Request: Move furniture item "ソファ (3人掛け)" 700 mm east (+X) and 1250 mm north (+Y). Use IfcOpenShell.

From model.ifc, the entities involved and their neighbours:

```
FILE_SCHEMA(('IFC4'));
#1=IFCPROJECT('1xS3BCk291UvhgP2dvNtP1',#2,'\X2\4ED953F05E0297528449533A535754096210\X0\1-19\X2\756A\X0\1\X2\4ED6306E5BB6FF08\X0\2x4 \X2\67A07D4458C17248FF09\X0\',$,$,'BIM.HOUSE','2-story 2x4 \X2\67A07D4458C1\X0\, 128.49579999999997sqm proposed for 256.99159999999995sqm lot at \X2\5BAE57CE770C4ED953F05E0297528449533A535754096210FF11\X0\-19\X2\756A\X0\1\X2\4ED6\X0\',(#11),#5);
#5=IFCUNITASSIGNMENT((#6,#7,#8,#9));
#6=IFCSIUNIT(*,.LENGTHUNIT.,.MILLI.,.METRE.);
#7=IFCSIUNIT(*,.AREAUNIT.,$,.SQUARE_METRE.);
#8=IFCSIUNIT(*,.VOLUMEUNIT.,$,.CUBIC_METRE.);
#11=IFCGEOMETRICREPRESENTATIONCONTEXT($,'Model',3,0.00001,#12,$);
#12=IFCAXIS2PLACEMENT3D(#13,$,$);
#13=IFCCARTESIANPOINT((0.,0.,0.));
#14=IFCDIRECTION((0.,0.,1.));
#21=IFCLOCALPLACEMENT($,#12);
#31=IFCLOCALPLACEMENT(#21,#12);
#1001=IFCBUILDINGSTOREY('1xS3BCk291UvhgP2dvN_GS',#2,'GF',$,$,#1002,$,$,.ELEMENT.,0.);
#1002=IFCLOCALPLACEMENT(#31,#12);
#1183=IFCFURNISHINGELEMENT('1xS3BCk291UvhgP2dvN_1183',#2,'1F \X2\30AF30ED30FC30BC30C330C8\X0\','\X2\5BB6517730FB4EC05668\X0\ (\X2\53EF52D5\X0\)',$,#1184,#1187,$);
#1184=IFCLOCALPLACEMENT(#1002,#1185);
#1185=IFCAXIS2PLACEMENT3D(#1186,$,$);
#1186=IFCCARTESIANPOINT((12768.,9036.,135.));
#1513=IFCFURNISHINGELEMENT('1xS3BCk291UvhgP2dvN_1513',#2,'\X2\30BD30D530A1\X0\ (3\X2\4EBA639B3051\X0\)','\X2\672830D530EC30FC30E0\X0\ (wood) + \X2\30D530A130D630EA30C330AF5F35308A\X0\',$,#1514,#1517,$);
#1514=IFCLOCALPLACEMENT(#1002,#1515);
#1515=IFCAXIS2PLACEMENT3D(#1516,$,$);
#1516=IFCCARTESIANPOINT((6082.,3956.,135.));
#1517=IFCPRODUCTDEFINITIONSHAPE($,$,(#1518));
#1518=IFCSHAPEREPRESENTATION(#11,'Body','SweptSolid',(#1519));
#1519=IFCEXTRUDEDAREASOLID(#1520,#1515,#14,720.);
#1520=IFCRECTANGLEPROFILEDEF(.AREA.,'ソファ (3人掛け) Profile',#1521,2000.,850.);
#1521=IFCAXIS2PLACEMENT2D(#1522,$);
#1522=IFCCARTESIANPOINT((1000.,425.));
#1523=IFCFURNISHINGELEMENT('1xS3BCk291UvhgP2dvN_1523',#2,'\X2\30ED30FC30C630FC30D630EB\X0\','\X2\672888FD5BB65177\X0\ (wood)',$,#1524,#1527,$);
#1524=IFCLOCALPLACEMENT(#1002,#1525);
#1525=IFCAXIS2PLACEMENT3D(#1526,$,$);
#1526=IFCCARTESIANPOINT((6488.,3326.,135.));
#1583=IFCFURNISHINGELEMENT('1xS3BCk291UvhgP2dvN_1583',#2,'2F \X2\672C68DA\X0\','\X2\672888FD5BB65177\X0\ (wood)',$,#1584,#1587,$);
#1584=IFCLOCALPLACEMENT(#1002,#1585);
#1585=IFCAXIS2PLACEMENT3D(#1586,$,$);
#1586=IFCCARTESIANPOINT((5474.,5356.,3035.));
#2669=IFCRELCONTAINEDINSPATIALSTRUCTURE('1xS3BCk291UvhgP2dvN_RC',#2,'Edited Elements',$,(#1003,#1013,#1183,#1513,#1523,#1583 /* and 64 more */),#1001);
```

```python
import ifcopenshell
import ifcopenshell.api.geometry
import ifcopenshell.util.placement
import ifcopenshell.util.unit

model = ifcopenshell.open("model.ifc")
unit_scale = ifcopenshell.util.unit.calculate_unit_scale(model)

item = model.by_guid("1xS3BCk291UvhgP2dvN_1513")
matrix = ifcopenshell.util.placement.get_local_placement(item.ObjectPlacement)
matrix[0, 3] += 0.7 / unit_scale
matrix[1, 3] += 1.25 / unit_scale
ifcopenshell.api.geometry.edit_object_placement(model, product=item, matrix=matrix, is_si=False)

print(ifcopenshell.util.placement.get_local_placement(item.ObjectPlacement).round(3) + 0.0)

model.write("model_v2.ifc")
```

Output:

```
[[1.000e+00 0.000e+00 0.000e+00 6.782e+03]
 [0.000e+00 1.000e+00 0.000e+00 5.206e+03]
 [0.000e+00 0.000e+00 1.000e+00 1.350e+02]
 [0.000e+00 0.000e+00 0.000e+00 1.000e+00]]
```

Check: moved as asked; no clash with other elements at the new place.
